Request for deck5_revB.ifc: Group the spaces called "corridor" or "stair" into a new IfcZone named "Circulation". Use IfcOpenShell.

First a look at what the model holds.

```python
import ifcopenshell

model = ifcopenshell.open("deck5_revB.ifc")
print(model.schema)
seen = {}
for space in model.by_type("IfcSpace"):
    seen[space.LongName] = seen.get(space.LongName, 0) + 1
for name, count in sorted(seen.items(), key=str):
    print(count, "x", name)
print("zones:", [z.Name for z in model.by_type("IfcZone")][:20])
```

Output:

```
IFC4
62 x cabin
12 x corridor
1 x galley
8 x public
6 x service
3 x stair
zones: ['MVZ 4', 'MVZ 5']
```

```python
import ifcopenshell
import ifcopenshell.api.group
import ifcopenshell.api.root

model = ifcopenshell.open("deck5_revB.ifc")

names = {"corridor", "stair"}
spaces = [s for s in model.by_type("IfcSpace") if s.LongName in names]

zone = ifcopenshell.api.root.create_entity(model, ifc_class="IfcZone", name="Circulation")
ifcopenshell.api.group.assign_group(model, products=spaces, group=zone)
print(len(spaces), "spaces in", zone.Name)

model.write("deck5_revB_rev.ifc")
```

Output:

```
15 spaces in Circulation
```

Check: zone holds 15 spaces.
